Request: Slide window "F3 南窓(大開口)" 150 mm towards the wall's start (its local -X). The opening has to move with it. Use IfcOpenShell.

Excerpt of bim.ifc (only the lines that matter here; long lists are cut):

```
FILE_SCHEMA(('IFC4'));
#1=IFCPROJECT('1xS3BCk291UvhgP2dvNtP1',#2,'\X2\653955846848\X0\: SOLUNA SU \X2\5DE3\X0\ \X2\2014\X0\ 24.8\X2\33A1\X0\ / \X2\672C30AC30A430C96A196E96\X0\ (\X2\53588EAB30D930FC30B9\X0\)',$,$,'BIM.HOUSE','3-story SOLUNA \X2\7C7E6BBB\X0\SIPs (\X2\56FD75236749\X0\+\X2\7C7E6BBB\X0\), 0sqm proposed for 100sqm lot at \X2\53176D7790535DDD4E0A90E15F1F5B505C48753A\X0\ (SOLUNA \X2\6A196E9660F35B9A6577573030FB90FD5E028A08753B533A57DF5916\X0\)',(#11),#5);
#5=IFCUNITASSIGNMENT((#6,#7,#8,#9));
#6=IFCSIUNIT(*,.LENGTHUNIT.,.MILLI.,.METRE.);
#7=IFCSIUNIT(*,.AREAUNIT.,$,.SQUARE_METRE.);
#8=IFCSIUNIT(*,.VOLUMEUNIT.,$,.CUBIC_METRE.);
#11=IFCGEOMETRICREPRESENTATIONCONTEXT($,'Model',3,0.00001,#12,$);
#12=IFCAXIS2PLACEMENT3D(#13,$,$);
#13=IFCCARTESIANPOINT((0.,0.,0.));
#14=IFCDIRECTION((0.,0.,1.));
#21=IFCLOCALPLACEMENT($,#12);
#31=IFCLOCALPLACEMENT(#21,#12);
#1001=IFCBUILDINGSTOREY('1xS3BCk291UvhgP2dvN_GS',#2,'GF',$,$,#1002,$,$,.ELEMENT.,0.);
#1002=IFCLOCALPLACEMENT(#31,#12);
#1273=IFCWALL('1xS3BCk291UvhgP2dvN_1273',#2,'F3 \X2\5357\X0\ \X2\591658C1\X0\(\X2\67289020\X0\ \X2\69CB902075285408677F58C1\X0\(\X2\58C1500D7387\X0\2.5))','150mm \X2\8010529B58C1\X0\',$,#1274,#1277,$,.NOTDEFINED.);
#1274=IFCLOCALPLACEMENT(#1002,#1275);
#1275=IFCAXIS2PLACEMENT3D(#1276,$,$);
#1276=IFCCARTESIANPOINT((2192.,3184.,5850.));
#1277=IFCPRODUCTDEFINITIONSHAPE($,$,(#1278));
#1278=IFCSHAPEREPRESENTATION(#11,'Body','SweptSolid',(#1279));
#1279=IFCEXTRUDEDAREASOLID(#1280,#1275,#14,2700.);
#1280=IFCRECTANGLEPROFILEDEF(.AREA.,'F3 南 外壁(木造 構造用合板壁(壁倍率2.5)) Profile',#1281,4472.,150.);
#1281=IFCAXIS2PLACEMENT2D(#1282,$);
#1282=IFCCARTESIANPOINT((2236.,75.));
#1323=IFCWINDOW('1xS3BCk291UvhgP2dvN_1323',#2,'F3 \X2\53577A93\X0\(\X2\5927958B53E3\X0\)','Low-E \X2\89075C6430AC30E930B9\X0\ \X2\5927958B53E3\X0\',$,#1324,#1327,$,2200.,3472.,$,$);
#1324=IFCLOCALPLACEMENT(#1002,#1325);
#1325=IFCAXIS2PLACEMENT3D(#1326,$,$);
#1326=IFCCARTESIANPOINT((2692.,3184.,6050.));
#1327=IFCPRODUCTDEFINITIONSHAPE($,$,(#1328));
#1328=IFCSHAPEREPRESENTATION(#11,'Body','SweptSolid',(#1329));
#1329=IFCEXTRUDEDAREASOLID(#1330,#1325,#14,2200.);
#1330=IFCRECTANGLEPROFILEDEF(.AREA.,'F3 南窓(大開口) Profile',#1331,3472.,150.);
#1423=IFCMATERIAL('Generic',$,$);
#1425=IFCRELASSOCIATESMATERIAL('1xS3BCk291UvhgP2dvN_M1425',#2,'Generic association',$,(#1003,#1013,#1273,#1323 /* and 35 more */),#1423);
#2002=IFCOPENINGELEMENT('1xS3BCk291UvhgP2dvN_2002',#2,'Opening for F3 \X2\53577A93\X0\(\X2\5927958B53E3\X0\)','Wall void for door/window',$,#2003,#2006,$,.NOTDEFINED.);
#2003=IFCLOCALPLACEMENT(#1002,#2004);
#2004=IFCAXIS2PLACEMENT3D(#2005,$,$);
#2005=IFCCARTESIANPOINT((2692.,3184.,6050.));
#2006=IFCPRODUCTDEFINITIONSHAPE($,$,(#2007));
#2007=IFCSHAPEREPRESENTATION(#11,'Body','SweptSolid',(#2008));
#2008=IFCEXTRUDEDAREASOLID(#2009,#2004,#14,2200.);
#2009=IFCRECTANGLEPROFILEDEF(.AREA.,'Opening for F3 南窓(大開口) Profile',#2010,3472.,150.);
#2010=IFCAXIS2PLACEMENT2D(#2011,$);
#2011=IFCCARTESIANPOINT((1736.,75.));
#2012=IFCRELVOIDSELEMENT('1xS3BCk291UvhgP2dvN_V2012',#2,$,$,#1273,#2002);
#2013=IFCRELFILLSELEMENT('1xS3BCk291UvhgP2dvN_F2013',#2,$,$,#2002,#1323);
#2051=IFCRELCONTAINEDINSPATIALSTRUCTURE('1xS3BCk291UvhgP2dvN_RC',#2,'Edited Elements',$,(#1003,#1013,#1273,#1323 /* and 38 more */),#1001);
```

```python
import ifcopenshell
import ifcopenshell.api.geometry
import ifcopenshell.util.placement

model = ifcopenshell.open("bim.ifc")

window = model.by_id(1323)
opening = window.FillsVoids[0].RelatingOpeningElement
wall = opening.VoidsElements[0].RelatingBuildingElement

wall_matrix = ifcopenshell.util.placement.get_local_placement(wall.ObjectPlacement)
shift = wall_matrix[:3, 0] * -150.0
before = ifcopenshell.util.placement.get_local_placement(window.ObjectPlacement)[:3, 3].copy()

# The window is not placed relative to its opening, so move both.
for product in (opening, window):
    matrix = ifcopenshell.util.placement.get_local_placement(product.ObjectPlacement)
    matrix[:3, 3] += shift
    ifcopenshell.api.geometry.edit_object_placement(model, product=product, matrix=matrix, is_si=False)

after = ifcopenshell.util.placement.get_local_placement(window.ObjectPlacement)[:3, 3]
print("window moved by", (after - before).round(3) + 0.0)

model.write("bim_v2.ifc")
```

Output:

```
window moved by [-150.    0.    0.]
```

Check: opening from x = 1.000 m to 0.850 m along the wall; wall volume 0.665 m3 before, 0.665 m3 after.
